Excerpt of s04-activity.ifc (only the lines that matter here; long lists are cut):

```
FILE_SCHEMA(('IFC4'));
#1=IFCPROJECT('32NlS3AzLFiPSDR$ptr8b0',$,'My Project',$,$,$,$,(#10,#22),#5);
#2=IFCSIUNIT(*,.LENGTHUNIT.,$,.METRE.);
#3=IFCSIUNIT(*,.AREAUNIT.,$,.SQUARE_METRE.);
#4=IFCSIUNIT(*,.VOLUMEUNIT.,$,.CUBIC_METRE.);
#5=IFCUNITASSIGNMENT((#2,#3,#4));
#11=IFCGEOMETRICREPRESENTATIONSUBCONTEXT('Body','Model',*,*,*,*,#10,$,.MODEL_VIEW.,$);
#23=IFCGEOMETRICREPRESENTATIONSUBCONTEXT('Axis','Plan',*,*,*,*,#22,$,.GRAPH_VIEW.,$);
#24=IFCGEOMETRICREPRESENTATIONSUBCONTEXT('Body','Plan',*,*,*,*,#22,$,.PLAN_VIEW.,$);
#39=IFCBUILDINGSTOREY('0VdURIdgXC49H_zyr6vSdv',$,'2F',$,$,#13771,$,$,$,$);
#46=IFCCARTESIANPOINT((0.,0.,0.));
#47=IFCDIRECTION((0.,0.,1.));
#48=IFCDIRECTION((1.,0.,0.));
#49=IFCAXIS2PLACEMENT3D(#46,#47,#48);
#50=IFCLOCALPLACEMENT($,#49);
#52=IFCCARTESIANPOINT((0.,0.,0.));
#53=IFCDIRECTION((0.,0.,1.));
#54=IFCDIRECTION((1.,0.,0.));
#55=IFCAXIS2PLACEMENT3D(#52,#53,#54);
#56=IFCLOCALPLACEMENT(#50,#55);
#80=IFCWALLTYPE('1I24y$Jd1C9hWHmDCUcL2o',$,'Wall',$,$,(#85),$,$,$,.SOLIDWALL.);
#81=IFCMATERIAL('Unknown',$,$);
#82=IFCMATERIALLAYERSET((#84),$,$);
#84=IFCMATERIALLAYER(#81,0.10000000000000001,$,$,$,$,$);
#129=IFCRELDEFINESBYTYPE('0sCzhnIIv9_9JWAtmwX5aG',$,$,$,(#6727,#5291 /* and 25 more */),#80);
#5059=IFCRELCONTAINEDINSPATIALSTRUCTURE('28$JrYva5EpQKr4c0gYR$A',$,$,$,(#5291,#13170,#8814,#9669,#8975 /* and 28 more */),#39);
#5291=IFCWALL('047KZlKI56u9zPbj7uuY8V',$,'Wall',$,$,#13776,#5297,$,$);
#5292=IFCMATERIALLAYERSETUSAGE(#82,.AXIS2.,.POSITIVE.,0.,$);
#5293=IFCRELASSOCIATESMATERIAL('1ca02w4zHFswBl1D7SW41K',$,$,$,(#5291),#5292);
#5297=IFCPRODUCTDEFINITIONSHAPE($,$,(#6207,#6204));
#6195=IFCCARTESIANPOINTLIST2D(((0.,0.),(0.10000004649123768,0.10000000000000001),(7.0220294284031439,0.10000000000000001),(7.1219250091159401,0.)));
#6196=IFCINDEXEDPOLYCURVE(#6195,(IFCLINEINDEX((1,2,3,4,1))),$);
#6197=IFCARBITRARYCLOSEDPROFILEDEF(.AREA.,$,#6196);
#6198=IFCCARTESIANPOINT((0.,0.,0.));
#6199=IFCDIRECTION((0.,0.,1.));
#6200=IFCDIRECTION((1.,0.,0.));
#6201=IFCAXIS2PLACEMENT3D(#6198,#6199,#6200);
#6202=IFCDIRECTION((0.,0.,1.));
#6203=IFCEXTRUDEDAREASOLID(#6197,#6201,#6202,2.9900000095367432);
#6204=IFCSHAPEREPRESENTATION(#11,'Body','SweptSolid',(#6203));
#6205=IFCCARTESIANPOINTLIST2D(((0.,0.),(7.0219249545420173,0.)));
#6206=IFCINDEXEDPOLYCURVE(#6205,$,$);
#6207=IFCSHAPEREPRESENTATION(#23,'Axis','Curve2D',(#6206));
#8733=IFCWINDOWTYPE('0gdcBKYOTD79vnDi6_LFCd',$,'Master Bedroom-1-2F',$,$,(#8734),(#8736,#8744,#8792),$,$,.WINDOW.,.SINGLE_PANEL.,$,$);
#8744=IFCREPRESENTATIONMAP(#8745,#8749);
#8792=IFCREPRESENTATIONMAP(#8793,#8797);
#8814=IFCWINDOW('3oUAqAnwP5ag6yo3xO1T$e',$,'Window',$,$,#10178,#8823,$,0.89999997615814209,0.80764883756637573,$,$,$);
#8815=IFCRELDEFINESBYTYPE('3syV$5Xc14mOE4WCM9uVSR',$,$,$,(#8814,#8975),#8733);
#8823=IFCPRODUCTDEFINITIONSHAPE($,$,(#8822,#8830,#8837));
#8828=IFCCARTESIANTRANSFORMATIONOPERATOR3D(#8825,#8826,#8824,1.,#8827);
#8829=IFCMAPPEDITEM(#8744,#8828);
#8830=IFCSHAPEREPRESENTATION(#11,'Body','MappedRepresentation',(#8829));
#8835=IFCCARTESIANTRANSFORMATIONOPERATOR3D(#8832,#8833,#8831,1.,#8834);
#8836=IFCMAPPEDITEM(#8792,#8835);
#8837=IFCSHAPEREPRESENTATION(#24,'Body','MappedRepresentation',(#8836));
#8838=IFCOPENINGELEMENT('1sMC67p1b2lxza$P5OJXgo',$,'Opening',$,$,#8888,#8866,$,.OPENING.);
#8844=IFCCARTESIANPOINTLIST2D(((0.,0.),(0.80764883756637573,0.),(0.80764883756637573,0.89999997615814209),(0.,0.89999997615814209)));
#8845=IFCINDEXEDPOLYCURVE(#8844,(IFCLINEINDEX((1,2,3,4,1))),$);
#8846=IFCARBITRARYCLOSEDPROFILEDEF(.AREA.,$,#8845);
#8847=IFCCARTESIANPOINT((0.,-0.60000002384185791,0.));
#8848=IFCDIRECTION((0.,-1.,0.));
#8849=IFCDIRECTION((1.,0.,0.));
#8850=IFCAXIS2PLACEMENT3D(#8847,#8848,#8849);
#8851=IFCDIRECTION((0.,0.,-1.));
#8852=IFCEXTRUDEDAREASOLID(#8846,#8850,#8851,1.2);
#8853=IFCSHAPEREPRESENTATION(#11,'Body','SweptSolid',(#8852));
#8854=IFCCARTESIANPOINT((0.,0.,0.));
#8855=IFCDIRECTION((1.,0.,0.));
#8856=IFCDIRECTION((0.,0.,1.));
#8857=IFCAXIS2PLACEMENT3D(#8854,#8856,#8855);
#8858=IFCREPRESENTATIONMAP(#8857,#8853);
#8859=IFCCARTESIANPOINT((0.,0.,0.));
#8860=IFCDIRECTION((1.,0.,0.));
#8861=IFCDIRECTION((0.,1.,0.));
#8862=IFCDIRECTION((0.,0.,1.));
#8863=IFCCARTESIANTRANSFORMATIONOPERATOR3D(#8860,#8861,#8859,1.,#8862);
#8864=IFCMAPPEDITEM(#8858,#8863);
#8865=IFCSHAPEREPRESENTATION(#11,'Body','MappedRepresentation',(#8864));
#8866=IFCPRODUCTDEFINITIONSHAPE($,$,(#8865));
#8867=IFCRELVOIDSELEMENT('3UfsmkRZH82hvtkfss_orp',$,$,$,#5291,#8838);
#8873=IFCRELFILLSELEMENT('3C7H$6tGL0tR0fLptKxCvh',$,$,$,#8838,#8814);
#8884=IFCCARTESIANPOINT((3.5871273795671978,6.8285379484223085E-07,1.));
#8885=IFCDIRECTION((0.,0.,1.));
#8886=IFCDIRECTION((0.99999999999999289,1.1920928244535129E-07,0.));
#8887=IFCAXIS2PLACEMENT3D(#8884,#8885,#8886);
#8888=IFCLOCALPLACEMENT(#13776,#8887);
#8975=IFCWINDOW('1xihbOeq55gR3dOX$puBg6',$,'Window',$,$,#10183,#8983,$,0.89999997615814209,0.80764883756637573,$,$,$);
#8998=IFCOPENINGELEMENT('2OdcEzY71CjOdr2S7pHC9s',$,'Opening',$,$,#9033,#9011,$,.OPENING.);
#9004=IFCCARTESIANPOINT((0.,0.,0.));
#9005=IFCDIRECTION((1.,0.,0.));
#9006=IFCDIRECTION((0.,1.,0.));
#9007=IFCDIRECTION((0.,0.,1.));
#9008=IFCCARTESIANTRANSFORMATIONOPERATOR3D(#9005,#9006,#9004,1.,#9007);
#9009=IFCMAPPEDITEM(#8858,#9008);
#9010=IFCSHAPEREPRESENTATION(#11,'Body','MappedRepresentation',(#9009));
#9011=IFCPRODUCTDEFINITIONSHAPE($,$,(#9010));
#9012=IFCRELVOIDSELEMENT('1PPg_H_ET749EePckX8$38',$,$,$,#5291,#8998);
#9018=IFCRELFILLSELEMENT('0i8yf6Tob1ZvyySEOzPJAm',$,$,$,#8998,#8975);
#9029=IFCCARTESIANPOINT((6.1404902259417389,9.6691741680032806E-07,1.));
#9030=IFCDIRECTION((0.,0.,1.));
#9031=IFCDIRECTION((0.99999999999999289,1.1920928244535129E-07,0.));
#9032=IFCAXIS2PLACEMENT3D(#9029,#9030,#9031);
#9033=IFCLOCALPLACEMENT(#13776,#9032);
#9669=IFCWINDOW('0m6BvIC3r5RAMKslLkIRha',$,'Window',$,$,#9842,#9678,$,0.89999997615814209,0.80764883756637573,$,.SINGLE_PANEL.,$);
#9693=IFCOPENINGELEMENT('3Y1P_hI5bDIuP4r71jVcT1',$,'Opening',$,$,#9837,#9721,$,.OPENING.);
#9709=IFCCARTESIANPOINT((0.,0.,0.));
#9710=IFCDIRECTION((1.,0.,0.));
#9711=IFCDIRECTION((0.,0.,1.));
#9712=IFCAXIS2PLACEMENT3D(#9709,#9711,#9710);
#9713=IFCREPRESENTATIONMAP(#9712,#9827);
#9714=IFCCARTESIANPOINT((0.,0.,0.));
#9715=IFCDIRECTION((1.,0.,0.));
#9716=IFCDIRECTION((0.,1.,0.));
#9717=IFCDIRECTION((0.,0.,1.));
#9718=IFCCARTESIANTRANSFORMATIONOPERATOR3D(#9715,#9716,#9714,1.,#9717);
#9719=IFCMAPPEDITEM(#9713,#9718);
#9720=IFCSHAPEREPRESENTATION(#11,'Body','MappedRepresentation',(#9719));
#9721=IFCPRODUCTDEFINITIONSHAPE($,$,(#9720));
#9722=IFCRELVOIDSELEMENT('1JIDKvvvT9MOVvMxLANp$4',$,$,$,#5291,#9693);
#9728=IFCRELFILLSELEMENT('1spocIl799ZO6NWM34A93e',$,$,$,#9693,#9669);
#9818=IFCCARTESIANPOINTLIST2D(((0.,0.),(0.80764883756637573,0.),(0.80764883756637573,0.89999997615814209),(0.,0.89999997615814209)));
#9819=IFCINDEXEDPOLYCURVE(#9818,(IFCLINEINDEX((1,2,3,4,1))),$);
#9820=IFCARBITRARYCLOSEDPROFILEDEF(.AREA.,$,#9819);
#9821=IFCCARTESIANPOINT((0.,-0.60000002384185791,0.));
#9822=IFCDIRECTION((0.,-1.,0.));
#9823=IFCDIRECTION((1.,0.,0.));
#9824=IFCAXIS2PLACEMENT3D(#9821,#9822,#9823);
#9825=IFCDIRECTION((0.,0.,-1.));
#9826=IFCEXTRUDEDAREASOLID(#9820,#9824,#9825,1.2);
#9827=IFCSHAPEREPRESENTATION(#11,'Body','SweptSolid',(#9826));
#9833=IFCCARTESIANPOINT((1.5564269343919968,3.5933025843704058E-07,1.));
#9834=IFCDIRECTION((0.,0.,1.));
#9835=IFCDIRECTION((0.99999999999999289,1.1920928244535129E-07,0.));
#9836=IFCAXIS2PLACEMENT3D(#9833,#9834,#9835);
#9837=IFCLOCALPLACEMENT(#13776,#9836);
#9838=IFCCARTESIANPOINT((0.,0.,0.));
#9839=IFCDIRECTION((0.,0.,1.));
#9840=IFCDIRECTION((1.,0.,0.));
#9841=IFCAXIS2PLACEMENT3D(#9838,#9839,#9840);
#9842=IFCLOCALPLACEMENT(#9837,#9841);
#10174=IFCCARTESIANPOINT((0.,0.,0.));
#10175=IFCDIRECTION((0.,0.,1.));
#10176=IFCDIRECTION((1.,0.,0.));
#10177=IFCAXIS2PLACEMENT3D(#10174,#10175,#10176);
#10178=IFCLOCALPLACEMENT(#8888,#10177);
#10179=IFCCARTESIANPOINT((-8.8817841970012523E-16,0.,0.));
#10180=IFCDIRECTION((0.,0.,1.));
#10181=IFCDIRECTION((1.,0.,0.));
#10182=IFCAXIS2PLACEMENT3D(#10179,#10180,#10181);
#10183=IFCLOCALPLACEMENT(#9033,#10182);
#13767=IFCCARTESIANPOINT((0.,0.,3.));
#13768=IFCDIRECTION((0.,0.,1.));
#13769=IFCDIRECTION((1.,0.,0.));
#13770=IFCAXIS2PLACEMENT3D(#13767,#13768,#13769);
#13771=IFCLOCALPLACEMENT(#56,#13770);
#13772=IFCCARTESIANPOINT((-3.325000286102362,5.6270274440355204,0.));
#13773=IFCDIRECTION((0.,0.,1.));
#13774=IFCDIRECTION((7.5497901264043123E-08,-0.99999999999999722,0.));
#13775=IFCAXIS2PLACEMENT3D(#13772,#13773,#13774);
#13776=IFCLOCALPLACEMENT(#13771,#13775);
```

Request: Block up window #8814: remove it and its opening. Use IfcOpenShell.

```python
import ifcopenshell
import ifcopenshell.api.feature
import ifcopenshell.api.root
import ifcopenshell.geom
import ifcopenshell.util.shape

model = ifcopenshell.open("s04-activity.ifc")
settings = ifcopenshell.geom.settings()


def volume(element):
    """Net volume in cubic metres, openings subtracted."""
    shape = ifcopenshell.geom.create_shape(settings, element)
    return ifcopenshell.util.shape.get_volume(shape.geometry)


window = model.by_guid("3oUAqAnwP5ag6yo3xO1T$e")
opening = window.FillsVoids[0].RelatingOpeningElement
wall = opening.VoidsElements[0].RelatingBuildingElement
before = volume(wall)

ifcopenshell.api.root.remove_product(model, product=window)
ifcopenshell.api.feature.remove_feature(model, feature=opening)

after = volume(wall)

print(f"wall volume {before:.3f} -> {after:.3f} m3")

model.write("s04-activity_edited.ifc")
```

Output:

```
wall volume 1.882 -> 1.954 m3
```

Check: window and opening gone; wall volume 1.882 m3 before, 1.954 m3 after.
